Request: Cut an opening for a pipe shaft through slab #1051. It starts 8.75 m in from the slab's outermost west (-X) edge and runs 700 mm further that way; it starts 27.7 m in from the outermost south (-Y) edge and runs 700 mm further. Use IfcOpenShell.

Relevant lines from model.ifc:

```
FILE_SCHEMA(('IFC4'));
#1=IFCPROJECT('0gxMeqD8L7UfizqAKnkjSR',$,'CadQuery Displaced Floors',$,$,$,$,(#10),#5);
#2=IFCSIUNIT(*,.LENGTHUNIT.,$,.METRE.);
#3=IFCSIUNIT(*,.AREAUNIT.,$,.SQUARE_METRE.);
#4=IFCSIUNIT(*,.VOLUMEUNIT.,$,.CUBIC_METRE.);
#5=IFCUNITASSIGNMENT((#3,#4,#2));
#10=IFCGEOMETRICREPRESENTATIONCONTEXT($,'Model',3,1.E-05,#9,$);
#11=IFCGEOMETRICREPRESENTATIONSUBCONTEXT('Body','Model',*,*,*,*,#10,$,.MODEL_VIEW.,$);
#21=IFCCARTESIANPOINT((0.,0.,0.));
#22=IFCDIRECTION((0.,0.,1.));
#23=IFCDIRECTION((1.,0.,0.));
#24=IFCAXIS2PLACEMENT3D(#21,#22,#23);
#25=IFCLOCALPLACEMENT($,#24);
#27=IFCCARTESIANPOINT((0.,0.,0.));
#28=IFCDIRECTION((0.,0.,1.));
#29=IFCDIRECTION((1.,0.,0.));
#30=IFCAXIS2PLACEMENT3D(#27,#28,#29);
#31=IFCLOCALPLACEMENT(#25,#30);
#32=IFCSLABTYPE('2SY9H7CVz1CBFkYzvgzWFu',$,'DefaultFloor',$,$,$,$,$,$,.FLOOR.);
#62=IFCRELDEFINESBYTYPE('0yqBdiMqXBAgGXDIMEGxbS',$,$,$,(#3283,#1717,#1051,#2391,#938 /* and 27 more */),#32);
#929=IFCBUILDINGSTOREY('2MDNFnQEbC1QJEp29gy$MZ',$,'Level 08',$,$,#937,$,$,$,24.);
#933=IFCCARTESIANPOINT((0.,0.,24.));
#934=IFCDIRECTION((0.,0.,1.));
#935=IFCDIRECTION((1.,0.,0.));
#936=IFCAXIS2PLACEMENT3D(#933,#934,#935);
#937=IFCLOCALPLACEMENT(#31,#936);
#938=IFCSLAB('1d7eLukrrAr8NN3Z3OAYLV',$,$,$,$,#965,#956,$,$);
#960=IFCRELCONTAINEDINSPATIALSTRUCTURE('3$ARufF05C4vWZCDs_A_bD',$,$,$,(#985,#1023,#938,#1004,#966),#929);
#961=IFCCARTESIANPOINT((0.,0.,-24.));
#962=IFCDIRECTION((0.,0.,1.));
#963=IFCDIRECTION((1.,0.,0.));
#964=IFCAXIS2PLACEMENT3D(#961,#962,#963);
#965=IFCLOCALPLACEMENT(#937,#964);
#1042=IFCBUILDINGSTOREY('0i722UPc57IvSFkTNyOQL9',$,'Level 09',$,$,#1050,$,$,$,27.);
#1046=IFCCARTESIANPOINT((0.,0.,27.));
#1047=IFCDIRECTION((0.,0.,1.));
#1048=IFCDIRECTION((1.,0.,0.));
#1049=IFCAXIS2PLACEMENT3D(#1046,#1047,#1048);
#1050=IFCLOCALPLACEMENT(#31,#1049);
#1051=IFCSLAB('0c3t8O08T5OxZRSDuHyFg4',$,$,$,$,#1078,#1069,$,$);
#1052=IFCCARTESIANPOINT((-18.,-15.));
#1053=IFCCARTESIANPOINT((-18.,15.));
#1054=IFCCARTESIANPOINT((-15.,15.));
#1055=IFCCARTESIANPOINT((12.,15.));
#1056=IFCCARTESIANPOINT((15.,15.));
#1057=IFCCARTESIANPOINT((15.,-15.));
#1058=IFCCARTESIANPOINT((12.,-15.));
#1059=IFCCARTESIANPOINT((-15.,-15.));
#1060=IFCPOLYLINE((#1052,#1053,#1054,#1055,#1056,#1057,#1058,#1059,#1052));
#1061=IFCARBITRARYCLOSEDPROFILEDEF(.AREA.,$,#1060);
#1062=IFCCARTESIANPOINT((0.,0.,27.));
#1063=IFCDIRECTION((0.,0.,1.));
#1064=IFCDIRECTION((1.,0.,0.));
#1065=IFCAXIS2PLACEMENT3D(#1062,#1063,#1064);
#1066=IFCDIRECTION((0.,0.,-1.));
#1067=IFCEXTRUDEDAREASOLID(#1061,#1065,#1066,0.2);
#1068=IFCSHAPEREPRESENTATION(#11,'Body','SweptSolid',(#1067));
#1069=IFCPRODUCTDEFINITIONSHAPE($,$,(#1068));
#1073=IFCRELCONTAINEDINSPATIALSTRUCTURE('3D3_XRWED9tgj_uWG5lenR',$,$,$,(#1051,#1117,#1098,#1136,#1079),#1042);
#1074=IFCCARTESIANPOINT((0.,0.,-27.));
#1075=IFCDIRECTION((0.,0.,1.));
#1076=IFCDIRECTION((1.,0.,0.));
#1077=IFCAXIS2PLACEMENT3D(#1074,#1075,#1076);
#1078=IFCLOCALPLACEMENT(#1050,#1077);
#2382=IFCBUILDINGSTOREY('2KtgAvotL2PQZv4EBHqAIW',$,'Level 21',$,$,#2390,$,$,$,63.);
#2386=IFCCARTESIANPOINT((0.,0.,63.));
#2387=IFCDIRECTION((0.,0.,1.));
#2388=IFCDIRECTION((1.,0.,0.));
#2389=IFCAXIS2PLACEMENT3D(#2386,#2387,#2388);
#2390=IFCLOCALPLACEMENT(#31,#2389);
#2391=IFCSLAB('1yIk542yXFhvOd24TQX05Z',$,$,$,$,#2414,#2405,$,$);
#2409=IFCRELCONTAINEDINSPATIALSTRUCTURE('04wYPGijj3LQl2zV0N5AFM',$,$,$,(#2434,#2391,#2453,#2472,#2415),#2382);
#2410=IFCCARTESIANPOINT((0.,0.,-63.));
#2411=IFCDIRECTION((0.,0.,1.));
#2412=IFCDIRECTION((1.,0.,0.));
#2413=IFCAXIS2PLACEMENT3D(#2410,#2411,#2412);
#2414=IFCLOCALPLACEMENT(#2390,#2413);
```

```python
import numpy as np
import ifcopenshell
import ifcopenshell.api.feature
import ifcopenshell.api.geometry
import ifcopenshell.api.root
import ifcopenshell.geom
import ifcopenshell.util.placement
import ifcopenshell.util.representation
import ifcopenshell.util.shape
import ifcopenshell.util.unit

model = ifcopenshell.open("model.ifc")
unit_scale = ifcopenshell.util.unit.calculate_unit_scale(model)
settings = ifcopenshell.geom.settings()


def volume(element):
    """Net volume in cubic metres, openings subtracted."""
    shape = ifcopenshell.geom.create_shape(settings, element)
    return ifcopenshell.util.shape.get_volume(shape.geometry)


slab = model.by_guid("0c3t8O08T5OxZRSDuHyFg4")
before = volume(slab)

# Extent in the slab's own axes, in metres. The edges named are its -X and -Y sides.
slab_shape = ifcopenshell.geom.create_shape(settings, slab)
vertices = ifcopenshell.util.shape.get_vertices(slab_shape.geometry)
x_min, y_min, bottom = vertices.min(axis=0)
top = vertices[:, 2].max()

opening = ifcopenshell.api.root.create_entity(model, ifc_class="IfcOpeningElement", name="Pipe shaft opening", predefined_type="OPENING")
context = ifcopenshell.util.representation.get_context(model, "Model", "Body", "MODEL_VIEW")
width, depth = 0.7, 0.7
outline = [(0.0, 0.0), (width, 0.0), (width, depth), (0.0, depth), (0.0, 0.0)]
# Overshoot both faces by 50 mm so the cut is clean.
shape = ifcopenshell.api.geometry.add_slab_representation(
    model, context=context, depth=top - bottom + 0.1, polyline=outline
)
ifcopenshell.api.geometry.assign_representation(model, product=opening, representation=shape)

matrix = ifcopenshell.util.placement.get_local_placement(slab.ObjectPlacement)
matrix[:, 3] = matrix @ np.append(np.array([x_min + 8.75, y_min + 27.7, bottom - 0.05]) / unit_scale, 1.0)
ifcopenshell.api.geometry.edit_object_placement(model, product=opening, matrix=matrix, is_si=False)
ifcopenshell.api.feature.add_feature(model, feature=opening, element=slab)

after = volume(slab)

print(f"slab volume {before:.3f} -> {after:.3f} m3")

model.write("model_updated.ifc")
```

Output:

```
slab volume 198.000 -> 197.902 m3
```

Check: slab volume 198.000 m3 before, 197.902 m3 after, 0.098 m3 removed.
